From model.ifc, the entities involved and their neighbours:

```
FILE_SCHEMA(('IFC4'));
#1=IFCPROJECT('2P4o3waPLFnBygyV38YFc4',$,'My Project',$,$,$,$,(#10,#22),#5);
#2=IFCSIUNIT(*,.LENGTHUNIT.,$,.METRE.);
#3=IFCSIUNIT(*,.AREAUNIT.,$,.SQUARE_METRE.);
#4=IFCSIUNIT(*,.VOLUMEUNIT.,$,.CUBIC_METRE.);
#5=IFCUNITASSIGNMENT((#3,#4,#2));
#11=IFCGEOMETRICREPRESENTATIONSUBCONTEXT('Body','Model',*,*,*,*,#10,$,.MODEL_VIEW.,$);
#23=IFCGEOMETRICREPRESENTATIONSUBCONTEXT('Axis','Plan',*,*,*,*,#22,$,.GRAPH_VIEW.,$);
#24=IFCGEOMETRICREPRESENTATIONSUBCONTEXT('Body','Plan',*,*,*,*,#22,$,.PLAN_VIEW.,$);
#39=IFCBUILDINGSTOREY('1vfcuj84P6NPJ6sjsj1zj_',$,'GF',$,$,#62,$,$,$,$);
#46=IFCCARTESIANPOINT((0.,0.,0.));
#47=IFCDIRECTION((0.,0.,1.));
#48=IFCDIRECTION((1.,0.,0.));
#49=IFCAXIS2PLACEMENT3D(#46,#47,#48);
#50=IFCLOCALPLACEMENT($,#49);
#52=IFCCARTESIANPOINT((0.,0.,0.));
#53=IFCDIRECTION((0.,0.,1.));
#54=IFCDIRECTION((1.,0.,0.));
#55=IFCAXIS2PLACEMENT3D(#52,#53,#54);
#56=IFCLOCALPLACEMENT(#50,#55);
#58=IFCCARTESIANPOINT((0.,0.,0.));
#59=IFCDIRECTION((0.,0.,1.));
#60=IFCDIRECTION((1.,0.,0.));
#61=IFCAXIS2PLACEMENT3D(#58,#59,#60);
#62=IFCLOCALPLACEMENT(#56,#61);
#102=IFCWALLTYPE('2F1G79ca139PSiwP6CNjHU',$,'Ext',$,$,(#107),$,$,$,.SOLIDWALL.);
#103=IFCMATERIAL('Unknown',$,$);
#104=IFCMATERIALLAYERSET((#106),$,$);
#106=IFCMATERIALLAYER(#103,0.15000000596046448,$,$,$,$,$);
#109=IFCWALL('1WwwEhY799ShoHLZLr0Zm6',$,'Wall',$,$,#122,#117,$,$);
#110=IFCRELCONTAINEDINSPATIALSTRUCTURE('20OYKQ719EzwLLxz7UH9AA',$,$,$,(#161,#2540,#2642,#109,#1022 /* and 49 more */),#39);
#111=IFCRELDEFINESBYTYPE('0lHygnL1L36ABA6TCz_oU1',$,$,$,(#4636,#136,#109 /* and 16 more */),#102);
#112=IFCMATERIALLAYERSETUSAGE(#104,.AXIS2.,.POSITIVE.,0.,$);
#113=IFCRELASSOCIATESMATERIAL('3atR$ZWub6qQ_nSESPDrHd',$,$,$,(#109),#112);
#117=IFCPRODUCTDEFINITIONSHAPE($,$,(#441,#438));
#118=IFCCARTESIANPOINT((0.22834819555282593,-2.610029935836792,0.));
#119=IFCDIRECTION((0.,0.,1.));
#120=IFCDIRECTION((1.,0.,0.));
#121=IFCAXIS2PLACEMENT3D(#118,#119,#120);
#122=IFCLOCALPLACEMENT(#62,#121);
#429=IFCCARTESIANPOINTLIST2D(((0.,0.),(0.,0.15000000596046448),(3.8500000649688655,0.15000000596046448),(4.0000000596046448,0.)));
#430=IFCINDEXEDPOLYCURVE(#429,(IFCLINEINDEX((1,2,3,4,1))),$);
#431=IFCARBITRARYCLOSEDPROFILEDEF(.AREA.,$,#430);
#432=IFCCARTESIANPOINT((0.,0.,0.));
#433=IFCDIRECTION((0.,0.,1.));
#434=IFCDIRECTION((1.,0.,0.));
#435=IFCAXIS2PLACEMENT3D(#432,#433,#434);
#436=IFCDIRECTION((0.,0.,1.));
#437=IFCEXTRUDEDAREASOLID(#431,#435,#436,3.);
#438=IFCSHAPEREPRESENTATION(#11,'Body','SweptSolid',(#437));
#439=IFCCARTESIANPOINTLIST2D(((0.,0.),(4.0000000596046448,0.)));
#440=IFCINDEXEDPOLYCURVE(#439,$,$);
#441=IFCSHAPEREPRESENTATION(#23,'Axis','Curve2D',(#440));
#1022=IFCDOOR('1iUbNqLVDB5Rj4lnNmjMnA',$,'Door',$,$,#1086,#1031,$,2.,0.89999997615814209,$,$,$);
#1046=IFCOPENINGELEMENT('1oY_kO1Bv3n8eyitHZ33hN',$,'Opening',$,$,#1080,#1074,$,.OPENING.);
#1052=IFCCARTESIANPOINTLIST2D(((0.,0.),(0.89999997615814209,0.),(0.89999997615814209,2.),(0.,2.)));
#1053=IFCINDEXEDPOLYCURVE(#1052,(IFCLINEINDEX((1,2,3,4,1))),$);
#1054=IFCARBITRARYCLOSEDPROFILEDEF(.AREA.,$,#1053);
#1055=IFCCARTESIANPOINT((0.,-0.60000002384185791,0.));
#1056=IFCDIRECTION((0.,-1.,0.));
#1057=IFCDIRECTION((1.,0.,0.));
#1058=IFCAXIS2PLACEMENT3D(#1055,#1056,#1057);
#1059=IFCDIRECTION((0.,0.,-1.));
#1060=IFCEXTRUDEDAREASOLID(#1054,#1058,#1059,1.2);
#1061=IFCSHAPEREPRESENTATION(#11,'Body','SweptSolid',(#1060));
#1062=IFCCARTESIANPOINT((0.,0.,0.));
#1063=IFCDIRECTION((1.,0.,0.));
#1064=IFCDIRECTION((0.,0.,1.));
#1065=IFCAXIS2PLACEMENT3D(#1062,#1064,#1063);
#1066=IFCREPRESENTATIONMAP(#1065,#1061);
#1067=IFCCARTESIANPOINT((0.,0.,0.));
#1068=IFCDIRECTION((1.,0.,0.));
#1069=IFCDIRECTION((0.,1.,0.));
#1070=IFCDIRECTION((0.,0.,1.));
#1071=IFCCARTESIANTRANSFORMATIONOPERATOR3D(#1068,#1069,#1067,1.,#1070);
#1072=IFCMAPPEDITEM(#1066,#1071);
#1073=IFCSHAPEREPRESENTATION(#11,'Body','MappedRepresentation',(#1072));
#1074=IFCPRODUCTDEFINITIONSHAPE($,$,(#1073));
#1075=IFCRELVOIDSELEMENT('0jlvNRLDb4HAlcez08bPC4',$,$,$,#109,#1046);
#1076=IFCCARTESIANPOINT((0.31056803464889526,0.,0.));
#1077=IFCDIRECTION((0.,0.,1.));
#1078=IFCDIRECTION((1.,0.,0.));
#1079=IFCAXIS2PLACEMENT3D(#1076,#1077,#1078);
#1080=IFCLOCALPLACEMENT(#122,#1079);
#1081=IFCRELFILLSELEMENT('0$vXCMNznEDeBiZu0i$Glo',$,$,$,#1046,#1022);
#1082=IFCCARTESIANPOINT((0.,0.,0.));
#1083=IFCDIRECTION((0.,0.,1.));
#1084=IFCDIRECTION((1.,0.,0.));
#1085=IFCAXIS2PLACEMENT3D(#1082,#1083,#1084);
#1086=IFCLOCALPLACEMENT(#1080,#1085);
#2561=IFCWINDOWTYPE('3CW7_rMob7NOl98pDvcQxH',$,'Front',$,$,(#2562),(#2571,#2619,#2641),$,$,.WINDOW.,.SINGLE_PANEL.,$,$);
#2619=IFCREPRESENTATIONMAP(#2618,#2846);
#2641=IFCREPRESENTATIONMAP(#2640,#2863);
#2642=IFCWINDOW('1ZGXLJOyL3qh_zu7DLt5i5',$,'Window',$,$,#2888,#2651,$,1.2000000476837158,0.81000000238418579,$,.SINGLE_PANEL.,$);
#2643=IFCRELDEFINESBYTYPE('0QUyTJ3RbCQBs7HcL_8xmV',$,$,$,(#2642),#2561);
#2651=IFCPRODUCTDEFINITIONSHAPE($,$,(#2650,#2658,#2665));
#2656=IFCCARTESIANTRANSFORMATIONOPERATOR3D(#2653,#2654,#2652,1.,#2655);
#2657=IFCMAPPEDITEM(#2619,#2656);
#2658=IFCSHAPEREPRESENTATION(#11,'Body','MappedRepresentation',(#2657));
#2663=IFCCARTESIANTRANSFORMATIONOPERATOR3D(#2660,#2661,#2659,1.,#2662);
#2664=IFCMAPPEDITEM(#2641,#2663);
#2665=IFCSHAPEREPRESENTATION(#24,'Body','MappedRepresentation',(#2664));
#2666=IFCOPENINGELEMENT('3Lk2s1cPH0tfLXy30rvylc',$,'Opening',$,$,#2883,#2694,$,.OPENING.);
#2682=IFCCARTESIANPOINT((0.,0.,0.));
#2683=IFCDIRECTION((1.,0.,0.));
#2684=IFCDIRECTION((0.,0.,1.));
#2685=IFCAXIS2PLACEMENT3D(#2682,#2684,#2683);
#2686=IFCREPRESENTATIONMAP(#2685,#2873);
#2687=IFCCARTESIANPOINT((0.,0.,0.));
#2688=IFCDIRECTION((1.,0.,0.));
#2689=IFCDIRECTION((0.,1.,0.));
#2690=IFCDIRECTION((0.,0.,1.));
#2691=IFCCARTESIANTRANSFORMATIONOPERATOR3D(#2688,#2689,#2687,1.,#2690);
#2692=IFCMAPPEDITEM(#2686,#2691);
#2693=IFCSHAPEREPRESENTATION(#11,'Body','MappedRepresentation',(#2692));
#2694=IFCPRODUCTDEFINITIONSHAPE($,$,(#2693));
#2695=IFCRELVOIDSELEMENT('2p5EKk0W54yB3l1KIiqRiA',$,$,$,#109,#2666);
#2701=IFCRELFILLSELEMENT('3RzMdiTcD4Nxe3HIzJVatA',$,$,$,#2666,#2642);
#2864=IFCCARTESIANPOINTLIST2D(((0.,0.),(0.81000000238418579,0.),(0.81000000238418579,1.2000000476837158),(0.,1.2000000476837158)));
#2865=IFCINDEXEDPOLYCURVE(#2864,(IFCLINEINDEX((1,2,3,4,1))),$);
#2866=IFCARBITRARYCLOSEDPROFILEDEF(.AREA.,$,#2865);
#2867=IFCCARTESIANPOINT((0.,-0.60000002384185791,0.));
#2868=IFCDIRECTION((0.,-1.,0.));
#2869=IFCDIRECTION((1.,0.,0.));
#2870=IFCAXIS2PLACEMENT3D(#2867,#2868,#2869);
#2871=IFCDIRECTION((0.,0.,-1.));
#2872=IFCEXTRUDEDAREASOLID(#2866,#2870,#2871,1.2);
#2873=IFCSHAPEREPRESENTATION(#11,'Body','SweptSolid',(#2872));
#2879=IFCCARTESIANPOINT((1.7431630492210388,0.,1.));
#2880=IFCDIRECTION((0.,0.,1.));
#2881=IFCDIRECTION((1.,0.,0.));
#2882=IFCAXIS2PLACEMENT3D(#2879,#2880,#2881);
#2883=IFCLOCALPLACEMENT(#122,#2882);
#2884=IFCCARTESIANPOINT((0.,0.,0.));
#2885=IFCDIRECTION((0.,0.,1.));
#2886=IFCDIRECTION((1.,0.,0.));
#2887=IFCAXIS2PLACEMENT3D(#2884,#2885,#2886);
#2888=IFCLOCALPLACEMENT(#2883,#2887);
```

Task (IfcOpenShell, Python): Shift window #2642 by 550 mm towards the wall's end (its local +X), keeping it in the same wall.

```python
import ifcopenshell
import ifcopenshell.api.geometry
import ifcopenshell.util.placement

model = ifcopenshell.open("model.ifc")

window = model.by_guid("1ZGXLJOyL3qh_zu7DLt5i5")
opening = window.FillsVoids[0].RelatingOpeningElement
wall = opening.VoidsElements[0].RelatingBuildingElement

wall_matrix = ifcopenshell.util.placement.get_local_placement(wall.ObjectPlacement)
shift = wall_matrix[:3, 0] * 0.55
before = ifcopenshell.util.placement.get_local_placement(window.ObjectPlacement)[:3, 3].copy()

# The window is placed relative to its opening, so it follows when the opening moves.
matrix = ifcopenshell.util.placement.get_local_placement(opening.ObjectPlacement)
matrix[:3, 3] += shift
ifcopenshell.api.geometry.edit_object_placement(
    model, product=opening, matrix=matrix, is_si=False, should_transform_children=True
)

after = ifcopenshell.util.placement.get_local_placement(window.ObjectPlacement)[:3, 3]
print("window moved by", (after - before).round(3) + 0.0)

model.write("model_v2.ifc")
```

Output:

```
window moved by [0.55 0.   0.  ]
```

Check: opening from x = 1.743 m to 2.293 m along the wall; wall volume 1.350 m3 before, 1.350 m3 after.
